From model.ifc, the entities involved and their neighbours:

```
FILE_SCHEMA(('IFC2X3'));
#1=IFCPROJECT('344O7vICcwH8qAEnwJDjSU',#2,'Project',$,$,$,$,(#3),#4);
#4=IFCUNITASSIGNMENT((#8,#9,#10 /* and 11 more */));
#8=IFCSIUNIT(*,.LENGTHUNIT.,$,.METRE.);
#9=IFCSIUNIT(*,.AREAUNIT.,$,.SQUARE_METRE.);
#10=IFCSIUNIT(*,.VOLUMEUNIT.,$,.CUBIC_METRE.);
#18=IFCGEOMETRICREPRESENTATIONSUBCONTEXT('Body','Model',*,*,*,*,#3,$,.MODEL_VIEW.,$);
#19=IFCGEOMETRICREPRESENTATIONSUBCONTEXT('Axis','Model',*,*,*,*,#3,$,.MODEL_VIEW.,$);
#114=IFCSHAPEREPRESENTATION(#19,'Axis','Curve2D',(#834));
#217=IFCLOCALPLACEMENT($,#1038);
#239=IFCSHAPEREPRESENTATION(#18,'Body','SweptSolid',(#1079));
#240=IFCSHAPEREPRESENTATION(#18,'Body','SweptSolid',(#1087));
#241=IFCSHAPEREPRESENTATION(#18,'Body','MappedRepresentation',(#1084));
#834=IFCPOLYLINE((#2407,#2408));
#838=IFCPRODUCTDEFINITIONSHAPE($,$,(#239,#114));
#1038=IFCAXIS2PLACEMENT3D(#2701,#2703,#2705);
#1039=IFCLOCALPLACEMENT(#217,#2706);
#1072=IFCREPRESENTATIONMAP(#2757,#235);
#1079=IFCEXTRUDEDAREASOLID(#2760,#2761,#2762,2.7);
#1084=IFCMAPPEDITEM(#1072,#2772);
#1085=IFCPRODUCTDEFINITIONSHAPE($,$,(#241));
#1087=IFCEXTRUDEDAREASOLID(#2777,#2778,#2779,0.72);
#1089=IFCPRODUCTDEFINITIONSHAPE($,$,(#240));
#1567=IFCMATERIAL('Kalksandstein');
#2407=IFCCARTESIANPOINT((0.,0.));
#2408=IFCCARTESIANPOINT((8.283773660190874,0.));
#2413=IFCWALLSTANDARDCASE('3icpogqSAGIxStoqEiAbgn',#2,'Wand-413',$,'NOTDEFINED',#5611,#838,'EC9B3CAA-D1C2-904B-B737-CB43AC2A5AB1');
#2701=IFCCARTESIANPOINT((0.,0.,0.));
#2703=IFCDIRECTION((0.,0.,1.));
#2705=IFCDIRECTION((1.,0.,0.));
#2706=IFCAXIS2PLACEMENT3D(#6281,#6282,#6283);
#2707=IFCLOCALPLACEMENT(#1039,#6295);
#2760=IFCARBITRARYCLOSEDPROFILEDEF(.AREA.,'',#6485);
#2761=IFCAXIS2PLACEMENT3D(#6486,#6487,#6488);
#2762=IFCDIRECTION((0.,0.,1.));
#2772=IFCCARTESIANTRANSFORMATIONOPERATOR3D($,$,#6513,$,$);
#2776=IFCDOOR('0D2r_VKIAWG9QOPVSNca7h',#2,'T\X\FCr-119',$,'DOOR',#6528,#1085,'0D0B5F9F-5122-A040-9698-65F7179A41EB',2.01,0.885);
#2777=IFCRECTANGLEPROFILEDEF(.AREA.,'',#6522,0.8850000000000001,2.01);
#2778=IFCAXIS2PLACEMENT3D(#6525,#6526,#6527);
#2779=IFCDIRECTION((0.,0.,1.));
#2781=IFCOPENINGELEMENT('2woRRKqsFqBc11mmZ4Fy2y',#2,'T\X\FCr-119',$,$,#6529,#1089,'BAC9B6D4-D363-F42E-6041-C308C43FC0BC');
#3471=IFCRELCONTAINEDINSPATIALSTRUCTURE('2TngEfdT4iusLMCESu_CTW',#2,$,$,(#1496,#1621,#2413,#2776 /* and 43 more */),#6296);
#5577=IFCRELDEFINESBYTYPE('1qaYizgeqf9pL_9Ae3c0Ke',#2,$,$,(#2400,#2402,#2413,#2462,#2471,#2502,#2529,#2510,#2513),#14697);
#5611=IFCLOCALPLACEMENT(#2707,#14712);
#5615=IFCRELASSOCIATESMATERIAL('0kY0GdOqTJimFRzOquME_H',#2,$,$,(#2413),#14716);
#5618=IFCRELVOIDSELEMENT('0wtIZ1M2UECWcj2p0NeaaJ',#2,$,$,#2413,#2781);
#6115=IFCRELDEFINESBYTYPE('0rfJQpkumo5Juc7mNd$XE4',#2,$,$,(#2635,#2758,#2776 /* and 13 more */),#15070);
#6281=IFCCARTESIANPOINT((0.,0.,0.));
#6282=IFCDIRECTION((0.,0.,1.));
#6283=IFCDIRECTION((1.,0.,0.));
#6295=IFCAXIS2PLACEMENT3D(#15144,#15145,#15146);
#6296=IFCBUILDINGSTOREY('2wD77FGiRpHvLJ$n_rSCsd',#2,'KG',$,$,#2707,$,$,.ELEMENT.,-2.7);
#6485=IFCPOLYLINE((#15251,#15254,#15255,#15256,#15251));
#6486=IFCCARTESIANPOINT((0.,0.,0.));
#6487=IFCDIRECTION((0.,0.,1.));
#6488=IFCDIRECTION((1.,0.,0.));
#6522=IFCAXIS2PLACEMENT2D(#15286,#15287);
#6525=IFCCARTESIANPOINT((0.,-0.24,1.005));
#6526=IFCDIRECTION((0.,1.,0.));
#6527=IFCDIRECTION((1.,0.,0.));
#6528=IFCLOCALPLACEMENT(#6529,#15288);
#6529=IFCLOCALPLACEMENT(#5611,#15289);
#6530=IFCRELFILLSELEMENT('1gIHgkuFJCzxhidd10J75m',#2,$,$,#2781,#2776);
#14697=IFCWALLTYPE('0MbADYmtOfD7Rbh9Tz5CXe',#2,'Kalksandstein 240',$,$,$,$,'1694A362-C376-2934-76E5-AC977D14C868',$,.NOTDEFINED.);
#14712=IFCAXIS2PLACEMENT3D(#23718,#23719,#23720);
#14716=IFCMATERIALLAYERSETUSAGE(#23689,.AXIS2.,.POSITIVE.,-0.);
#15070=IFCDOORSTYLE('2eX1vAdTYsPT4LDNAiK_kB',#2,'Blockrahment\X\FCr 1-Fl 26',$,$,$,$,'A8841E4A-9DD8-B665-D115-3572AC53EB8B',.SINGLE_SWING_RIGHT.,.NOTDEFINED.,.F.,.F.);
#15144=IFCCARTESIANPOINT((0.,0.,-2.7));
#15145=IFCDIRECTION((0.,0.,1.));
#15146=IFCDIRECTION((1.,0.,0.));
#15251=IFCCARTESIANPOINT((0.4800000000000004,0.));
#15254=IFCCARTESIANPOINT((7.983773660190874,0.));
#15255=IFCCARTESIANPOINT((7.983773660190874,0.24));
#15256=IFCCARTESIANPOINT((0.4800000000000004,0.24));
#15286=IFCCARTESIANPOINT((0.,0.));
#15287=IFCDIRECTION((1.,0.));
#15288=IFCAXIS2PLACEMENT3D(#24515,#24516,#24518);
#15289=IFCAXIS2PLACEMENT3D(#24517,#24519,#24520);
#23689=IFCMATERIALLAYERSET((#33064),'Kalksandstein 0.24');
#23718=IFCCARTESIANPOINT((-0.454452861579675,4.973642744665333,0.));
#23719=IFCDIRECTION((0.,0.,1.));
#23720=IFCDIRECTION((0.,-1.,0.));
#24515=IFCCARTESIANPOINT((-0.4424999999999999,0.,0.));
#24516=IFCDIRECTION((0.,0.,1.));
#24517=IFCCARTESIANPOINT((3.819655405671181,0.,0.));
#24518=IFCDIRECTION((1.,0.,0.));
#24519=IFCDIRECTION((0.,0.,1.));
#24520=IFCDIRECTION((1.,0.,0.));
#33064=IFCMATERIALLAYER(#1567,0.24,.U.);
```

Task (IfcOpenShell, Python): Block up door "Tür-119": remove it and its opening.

```python
import ifcopenshell
import ifcopenshell.api.feature
import ifcopenshell.api.root
import ifcopenshell.geom
import ifcopenshell.util.shape

model = ifcopenshell.open("model.ifc")
settings = ifcopenshell.geom.settings()


def volume(element):
    """Net volume in cubic metres, openings subtracted."""
    shape = ifcopenshell.geom.create_shape(settings, element)
    return ifcopenshell.util.shape.get_volume(shape.geometry)


door = model.by_guid("0D2r_VKIAWG9QOPVSNca7h")
opening = door.FillsVoids[0].RelatingOpeningElement
wall = opening.VoidsElements[0].RelatingBuildingElement
before = volume(wall)

ifcopenshell.api.root.remove_product(model, product=door)
ifcopenshell.api.feature.remove_feature(model, feature=opening)

after = volume(wall)

print(f"wall volume {before:.3f} -> {after:.3f} m3")

model.write("model_updated.ifc")
```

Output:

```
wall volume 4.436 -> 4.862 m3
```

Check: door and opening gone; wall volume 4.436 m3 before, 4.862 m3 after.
